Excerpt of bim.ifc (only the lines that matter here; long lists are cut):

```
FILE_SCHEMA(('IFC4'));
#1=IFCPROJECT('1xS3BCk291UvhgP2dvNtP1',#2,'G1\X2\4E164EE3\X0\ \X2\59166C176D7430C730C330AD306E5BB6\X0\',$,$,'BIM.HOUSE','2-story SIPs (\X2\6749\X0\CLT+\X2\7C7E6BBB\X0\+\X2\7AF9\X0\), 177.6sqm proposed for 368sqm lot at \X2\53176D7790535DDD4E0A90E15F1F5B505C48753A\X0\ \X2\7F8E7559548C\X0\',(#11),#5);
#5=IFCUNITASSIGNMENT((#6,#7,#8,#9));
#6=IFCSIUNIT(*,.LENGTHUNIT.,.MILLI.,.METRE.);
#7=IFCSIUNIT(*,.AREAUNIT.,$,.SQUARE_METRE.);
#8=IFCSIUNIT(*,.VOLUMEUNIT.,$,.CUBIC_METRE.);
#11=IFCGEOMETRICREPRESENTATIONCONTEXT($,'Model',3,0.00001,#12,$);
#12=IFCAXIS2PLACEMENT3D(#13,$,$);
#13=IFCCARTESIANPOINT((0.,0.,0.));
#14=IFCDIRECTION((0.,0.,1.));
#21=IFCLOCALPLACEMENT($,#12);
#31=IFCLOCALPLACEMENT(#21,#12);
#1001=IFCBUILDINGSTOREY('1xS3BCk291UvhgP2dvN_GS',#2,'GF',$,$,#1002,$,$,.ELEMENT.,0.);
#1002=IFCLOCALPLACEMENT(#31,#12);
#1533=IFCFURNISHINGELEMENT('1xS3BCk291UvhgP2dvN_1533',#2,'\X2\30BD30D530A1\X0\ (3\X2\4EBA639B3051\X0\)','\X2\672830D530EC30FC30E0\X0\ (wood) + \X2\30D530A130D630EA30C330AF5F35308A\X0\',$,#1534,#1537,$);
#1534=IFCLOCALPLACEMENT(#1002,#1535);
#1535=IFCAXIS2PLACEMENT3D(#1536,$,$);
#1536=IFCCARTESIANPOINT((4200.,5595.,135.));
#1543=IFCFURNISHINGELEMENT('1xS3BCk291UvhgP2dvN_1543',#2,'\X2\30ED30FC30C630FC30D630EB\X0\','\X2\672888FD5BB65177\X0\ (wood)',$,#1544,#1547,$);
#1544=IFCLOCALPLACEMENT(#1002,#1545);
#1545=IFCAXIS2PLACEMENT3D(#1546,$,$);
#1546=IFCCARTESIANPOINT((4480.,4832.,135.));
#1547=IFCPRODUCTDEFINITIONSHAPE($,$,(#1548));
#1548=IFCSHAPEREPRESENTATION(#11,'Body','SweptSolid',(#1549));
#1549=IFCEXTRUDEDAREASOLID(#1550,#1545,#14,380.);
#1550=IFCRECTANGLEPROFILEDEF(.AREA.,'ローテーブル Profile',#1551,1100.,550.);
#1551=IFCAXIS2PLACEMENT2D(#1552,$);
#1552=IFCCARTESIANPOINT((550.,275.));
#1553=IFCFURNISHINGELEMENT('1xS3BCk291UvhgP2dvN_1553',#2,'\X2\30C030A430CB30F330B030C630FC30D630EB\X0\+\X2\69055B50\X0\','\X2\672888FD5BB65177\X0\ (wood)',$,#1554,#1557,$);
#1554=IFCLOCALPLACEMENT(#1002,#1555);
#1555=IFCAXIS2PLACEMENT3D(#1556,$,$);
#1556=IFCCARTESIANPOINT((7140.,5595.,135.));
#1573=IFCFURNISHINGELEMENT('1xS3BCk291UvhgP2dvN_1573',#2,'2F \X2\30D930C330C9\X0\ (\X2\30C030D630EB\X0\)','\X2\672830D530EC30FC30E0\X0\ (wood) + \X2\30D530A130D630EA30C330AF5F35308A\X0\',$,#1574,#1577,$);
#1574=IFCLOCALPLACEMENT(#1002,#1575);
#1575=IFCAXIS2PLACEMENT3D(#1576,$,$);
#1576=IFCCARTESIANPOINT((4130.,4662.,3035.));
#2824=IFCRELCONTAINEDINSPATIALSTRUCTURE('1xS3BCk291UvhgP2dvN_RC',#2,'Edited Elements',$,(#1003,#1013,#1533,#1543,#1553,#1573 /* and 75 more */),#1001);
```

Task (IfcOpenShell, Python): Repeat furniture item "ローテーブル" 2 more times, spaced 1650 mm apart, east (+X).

```python
import numpy as np
import ifcopenshell
import ifcopenshell.api.geometry
import ifcopenshell.api.root
import ifcopenshell.util.element
import ifcopenshell.util.placement

model = ifcopenshell.open("bim.ifc")


def reuse_history(source, copy):
    """copy_class also copies each property set's owner history, people and application; keep the originals."""
    for rel in copy.IsDefinedBy:
        if rel.is_a("IfcRelDefinesByProperties") and (history := rel.RelatingPropertyDefinition.OwnerHistory):
            rel.RelatingPropertyDefinition.OwnerHistory = source.OwnerHistory
            ifcopenshell.util.element.remove_deep2(model, history)


source = model.by_guid("1xS3BCk291UvhgP2dvN_1543")
base = ifcopenshell.util.placement.get_local_placement(source.ObjectPlacement)
step = np.array([1.0, 0.0, 0.0]) * 1650.0

for i in range(1, 3):
    copy = ifcopenshell.api.root.copy_class(model, product=source)
    copy.Representation = ifcopenshell.util.element.copy_deep(
        model, source.Representation, exclude=["IfcGeometricRepresentationContext", "IfcRepresentationMap"]
    )
    reuse_history(source, copy)
    matrix = base.copy()
    matrix[:3, 3] += i * step
    print("added at", matrix[:3, 3].round(3) + 0.0)
    ifcopenshell.api.geometry.edit_object_placement(model, product=copy, matrix=matrix, is_si=False)

model.write("bim_edited.ifc")
```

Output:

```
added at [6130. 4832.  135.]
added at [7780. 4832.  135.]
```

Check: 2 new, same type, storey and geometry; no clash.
